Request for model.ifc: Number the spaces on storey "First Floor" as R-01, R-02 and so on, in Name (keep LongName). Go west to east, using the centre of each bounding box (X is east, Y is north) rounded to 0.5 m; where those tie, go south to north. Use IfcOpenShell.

First a look at what the model holds.

```python
import ifcopenshell
import ifcopenshell.util.element
import ifcopenshell.util.placement

model = ifcopenshell.open("model.ifc")
print(model.schema)
storey = next(s for s in model.by_type("IfcBuildingStorey") if s.Name == "First Floor")
spaces = [e for e in ifcopenshell.util.element.get_decomposition(storey) if e.is_a("IfcSpace")]
for e in sorted(spaces, key=lambda e: e.id()):
    origin = ifcopenshell.util.placement.get_local_placement(e.ObjectPlacement)[:3, 3]
    print(e.id(), e.Name, e.LongName, origin.round(2) + 0.0, sep=" | ")
```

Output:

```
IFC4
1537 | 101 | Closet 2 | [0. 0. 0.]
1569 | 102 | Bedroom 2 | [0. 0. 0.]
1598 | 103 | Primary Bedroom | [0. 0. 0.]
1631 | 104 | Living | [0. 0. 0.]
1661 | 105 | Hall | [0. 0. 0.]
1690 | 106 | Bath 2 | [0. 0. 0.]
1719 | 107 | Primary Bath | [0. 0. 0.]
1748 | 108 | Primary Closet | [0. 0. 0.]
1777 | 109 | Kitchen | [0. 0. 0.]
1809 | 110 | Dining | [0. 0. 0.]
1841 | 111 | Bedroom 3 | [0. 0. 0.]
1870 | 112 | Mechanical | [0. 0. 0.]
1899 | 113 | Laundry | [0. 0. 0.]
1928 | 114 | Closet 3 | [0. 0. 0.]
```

```python
import ifcopenshell
import ifcopenshell.geom
import ifcopenshell.util.element
import ifcopenshell.util.shape

model = ifcopenshell.open("model.ifc")
settings = ifcopenshell.geom.settings()
settings.set("use-world-coords", True)


def centre(element):
    shape = ifcopenshell.geom.create_shape(settings, element)
    return ifcopenshell.util.shape.get_bbox_centroid(shape.geometry)


storey = next(s for s in model.by_type("IfcBuildingStorey") if s.Name == "First Floor")
spaces = [e for e in ifcopenshell.util.element.get_decomposition(storey) if e.is_a("IfcSpace")]

# Insertion points can sit at a corner or the storey origin, so sort by the geometry (in metres).
centres = {e: centre(e) for e in spaces}
spaces.sort(key=lambda e: (round(centres[e][0] / 0.5), centres[e][1]))

for i, e in enumerate(spaces, start=1):
    number = f"R-{i:02d}"
    e.Name = number
    print(e.id(), number)

model.write("model-out.ifc")
```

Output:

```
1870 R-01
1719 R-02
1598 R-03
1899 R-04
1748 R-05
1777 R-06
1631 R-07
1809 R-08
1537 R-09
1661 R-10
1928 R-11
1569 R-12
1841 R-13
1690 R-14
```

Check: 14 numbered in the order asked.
